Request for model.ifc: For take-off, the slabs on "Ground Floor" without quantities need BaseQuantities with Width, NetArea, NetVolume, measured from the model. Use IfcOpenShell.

First a look at what the model holds.

```python
import ifcopenshell
import ifcopenshell.util.element
import ifcopenshell.util.unit

model = ifcopenshell.open("model.ifc")
print(model.schema)
for unit_type in ("LENGTHUNIT", "AREAUNIT", "VOLUMEUNIT"):
    print(unit_type, ifcopenshell.util.unit.calculate_unit_scale(model, unit_type))
storey = next(s for s in model.by_type("IfcBuildingStorey") if s.Name == "Ground Floor")
slabs = [e for e in ifcopenshell.util.element.get_decomposition(storey) if e.is_a("IfcSlab")]
for e in sorted(slabs, key=lambda e: e.id()):
    print(e.id(), e.is_a(), e.Name, list(ifcopenshell.util.element.get_psets(e, qtos_only=True)), sep=" | ")
```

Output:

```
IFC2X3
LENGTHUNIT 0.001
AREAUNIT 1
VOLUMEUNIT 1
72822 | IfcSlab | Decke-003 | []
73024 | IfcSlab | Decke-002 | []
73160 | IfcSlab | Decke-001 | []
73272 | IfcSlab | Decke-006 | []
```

```python
import ifcopenshell
import ifcopenshell.api.pset
import ifcopenshell.geom
import ifcopenshell.util.element
import ifcopenshell.util.shape
import ifcopenshell.util.unit

model = ifcopenshell.open("model.ifc")
unit_scale = ifcopenshell.util.unit.calculate_unit_scale(model)
area_scale = ifcopenshell.util.unit.calculate_unit_scale(model, "AREAUNIT")
volume_scale = ifcopenshell.util.unit.calculate_unit_scale(model, "VOLUMEUNIT")
settings = ifcopenshell.geom.settings()

storey = next(s for s in model.by_type("IfcBuildingStorey") if s.Name == "Ground Floor")
slabs = [e for e in ifcopenshell.util.element.get_decomposition(storey) if e.is_a("IfcSlab")]

for e in sorted(slabs, key=lambda e: e.id()):
    if ifcopenshell.util.element.get_psets(e, qtos_only=True, should_inherit=False):
        continue
    # Geometry comes back in metres, in the element's own axes.
    shape = ifcopenshell.geom.create_shape(settings, e)
    values = {
        "Width": ifcopenshell.util.shape.get_z(shape.geometry) / unit_scale,
        "NetArea": ifcopenshell.util.shape.get_footprint_area(shape.geometry) / area_scale,
        "NetVolume": ifcopenshell.util.shape.get_volume(shape.geometry) / volume_scale,
    }
    qto = ifcopenshell.api.pset.add_qto(model, product=e, name="BaseQuantities")
    ifcopenshell.api.pset.edit_qto(model, qto=qto, properties=values)
    print(e.id(), {k: round(v, 3) for k, v in values.items()})

model.write("model_rev.ifc")
```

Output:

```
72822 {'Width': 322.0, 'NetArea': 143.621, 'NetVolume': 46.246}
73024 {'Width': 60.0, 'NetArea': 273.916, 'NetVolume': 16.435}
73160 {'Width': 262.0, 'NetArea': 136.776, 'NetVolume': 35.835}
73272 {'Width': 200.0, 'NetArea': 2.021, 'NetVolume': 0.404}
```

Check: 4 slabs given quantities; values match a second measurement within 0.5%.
